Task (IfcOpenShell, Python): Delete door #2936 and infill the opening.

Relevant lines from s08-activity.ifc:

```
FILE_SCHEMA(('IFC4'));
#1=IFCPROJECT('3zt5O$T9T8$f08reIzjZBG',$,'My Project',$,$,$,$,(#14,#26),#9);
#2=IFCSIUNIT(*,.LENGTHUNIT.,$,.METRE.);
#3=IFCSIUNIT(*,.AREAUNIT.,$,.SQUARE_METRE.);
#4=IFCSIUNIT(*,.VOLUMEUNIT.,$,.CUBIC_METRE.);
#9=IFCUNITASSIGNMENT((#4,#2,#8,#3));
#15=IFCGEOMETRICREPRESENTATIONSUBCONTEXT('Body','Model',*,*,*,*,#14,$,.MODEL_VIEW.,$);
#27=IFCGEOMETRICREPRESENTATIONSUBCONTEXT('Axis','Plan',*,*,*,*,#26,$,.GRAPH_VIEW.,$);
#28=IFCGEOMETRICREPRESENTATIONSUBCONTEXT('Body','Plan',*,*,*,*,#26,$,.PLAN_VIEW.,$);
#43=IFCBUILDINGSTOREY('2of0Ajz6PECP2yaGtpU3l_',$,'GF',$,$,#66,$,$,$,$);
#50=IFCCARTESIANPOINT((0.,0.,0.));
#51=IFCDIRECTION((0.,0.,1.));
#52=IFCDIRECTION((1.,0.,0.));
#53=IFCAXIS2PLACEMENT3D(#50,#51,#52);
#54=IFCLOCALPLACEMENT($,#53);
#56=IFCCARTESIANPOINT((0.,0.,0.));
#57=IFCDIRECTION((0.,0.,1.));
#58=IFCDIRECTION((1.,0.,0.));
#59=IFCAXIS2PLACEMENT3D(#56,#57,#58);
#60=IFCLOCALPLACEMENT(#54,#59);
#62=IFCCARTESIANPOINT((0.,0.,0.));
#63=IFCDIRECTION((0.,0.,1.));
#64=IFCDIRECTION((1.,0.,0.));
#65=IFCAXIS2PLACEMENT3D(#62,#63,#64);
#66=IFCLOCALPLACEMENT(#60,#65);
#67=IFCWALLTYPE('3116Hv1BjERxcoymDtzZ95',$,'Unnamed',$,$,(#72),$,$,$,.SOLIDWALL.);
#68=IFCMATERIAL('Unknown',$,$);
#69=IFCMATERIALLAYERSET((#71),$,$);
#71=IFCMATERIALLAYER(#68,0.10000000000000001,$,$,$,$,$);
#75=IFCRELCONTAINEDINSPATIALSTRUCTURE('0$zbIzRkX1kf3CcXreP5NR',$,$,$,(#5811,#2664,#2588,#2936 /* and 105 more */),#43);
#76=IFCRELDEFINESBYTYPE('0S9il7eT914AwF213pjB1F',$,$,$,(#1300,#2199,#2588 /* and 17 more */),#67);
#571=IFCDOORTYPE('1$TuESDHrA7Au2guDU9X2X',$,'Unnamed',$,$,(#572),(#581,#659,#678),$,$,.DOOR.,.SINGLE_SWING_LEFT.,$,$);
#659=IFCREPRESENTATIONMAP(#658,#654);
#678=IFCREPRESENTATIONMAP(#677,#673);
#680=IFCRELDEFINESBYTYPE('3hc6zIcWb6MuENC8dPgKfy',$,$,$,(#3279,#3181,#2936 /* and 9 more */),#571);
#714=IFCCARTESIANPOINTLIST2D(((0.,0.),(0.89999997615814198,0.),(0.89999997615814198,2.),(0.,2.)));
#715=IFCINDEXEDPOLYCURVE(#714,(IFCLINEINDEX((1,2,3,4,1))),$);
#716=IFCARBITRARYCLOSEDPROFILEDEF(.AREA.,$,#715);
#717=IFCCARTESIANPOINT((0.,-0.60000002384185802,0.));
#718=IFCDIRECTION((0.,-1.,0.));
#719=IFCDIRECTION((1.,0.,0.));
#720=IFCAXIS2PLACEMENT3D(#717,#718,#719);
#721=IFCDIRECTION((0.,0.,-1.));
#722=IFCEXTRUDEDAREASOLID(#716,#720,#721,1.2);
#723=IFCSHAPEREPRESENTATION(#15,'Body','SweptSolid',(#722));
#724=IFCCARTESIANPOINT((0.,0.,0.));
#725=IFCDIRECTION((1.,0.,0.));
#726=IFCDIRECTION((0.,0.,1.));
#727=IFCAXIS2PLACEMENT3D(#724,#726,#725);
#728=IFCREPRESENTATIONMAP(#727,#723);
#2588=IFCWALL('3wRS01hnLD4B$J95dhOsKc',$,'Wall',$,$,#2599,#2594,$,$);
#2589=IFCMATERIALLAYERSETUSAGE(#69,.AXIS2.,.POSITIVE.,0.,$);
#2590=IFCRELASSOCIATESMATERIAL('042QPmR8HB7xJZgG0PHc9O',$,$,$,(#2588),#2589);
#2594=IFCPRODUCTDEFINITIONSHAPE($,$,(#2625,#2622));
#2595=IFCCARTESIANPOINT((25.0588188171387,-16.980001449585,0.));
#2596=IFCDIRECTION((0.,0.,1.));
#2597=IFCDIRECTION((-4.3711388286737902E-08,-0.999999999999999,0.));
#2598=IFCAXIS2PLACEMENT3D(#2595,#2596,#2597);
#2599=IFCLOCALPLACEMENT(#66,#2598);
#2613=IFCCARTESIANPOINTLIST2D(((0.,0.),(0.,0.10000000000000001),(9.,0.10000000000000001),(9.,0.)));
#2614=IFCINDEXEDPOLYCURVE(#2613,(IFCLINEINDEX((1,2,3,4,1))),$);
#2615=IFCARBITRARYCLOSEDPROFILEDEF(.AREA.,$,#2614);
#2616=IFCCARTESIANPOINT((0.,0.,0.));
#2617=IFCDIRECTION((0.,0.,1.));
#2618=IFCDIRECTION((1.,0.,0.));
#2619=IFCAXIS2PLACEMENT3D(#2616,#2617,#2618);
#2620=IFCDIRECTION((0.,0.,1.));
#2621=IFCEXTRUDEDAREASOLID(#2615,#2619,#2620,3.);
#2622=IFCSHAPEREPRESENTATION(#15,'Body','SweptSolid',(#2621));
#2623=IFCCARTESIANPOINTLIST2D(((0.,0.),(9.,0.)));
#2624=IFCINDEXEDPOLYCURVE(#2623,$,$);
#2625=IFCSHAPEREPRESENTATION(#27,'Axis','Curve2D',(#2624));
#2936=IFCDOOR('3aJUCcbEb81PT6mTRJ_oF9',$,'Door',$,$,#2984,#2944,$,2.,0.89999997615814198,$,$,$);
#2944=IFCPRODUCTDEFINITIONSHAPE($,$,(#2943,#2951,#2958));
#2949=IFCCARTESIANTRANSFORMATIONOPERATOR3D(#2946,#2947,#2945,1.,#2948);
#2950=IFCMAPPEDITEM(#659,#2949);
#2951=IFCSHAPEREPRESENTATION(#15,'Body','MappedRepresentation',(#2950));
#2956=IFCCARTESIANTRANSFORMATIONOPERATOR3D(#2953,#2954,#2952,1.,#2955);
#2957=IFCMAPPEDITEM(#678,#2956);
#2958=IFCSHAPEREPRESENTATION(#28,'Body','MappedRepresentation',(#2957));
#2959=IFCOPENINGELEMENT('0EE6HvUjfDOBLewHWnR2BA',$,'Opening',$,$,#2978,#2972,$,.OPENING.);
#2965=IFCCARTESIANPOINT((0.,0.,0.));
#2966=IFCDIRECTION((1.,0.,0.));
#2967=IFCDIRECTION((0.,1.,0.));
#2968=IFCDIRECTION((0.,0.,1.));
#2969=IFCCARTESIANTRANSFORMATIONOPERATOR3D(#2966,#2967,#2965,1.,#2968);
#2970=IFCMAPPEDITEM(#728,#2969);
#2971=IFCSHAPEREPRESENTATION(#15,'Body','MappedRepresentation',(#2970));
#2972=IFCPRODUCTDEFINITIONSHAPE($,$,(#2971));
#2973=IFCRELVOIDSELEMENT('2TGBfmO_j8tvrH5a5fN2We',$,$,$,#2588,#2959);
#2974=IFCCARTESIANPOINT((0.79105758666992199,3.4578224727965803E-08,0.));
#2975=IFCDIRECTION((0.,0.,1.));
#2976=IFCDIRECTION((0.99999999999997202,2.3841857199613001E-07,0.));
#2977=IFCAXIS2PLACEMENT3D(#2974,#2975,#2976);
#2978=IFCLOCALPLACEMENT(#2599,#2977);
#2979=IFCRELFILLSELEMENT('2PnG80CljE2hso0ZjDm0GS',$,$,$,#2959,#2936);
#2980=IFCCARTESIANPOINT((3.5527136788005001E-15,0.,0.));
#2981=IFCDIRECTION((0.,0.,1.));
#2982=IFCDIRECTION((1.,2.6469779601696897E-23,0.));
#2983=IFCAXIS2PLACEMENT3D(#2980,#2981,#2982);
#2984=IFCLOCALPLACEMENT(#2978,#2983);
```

```python
import ifcopenshell
import ifcopenshell.api.feature
import ifcopenshell.api.root
import ifcopenshell.geom
import ifcopenshell.util.shape

model = ifcopenshell.open("s08-activity.ifc")
settings = ifcopenshell.geom.settings()


def volume(element):
    """Net volume in cubic metres, openings subtracted."""
    shape = ifcopenshell.geom.create_shape(settings, element)
    return ifcopenshell.util.shape.get_volume(shape.geometry)


door = model.by_guid("3aJUCcbEb81PT6mTRJ_oF9")
opening = door.FillsVoids[0].RelatingOpeningElement
wall = opening.VoidsElements[0].RelatingBuildingElement
before = volume(wall)

ifcopenshell.api.root.remove_product(model, product=door)
ifcopenshell.api.feature.remove_feature(model, feature=opening)

after = volume(wall)

print(f"wall volume {before:.3f} -> {after:.3f} m3")

model.write("s08-activity-out.ifc")
```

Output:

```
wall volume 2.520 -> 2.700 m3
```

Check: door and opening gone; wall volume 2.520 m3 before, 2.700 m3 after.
